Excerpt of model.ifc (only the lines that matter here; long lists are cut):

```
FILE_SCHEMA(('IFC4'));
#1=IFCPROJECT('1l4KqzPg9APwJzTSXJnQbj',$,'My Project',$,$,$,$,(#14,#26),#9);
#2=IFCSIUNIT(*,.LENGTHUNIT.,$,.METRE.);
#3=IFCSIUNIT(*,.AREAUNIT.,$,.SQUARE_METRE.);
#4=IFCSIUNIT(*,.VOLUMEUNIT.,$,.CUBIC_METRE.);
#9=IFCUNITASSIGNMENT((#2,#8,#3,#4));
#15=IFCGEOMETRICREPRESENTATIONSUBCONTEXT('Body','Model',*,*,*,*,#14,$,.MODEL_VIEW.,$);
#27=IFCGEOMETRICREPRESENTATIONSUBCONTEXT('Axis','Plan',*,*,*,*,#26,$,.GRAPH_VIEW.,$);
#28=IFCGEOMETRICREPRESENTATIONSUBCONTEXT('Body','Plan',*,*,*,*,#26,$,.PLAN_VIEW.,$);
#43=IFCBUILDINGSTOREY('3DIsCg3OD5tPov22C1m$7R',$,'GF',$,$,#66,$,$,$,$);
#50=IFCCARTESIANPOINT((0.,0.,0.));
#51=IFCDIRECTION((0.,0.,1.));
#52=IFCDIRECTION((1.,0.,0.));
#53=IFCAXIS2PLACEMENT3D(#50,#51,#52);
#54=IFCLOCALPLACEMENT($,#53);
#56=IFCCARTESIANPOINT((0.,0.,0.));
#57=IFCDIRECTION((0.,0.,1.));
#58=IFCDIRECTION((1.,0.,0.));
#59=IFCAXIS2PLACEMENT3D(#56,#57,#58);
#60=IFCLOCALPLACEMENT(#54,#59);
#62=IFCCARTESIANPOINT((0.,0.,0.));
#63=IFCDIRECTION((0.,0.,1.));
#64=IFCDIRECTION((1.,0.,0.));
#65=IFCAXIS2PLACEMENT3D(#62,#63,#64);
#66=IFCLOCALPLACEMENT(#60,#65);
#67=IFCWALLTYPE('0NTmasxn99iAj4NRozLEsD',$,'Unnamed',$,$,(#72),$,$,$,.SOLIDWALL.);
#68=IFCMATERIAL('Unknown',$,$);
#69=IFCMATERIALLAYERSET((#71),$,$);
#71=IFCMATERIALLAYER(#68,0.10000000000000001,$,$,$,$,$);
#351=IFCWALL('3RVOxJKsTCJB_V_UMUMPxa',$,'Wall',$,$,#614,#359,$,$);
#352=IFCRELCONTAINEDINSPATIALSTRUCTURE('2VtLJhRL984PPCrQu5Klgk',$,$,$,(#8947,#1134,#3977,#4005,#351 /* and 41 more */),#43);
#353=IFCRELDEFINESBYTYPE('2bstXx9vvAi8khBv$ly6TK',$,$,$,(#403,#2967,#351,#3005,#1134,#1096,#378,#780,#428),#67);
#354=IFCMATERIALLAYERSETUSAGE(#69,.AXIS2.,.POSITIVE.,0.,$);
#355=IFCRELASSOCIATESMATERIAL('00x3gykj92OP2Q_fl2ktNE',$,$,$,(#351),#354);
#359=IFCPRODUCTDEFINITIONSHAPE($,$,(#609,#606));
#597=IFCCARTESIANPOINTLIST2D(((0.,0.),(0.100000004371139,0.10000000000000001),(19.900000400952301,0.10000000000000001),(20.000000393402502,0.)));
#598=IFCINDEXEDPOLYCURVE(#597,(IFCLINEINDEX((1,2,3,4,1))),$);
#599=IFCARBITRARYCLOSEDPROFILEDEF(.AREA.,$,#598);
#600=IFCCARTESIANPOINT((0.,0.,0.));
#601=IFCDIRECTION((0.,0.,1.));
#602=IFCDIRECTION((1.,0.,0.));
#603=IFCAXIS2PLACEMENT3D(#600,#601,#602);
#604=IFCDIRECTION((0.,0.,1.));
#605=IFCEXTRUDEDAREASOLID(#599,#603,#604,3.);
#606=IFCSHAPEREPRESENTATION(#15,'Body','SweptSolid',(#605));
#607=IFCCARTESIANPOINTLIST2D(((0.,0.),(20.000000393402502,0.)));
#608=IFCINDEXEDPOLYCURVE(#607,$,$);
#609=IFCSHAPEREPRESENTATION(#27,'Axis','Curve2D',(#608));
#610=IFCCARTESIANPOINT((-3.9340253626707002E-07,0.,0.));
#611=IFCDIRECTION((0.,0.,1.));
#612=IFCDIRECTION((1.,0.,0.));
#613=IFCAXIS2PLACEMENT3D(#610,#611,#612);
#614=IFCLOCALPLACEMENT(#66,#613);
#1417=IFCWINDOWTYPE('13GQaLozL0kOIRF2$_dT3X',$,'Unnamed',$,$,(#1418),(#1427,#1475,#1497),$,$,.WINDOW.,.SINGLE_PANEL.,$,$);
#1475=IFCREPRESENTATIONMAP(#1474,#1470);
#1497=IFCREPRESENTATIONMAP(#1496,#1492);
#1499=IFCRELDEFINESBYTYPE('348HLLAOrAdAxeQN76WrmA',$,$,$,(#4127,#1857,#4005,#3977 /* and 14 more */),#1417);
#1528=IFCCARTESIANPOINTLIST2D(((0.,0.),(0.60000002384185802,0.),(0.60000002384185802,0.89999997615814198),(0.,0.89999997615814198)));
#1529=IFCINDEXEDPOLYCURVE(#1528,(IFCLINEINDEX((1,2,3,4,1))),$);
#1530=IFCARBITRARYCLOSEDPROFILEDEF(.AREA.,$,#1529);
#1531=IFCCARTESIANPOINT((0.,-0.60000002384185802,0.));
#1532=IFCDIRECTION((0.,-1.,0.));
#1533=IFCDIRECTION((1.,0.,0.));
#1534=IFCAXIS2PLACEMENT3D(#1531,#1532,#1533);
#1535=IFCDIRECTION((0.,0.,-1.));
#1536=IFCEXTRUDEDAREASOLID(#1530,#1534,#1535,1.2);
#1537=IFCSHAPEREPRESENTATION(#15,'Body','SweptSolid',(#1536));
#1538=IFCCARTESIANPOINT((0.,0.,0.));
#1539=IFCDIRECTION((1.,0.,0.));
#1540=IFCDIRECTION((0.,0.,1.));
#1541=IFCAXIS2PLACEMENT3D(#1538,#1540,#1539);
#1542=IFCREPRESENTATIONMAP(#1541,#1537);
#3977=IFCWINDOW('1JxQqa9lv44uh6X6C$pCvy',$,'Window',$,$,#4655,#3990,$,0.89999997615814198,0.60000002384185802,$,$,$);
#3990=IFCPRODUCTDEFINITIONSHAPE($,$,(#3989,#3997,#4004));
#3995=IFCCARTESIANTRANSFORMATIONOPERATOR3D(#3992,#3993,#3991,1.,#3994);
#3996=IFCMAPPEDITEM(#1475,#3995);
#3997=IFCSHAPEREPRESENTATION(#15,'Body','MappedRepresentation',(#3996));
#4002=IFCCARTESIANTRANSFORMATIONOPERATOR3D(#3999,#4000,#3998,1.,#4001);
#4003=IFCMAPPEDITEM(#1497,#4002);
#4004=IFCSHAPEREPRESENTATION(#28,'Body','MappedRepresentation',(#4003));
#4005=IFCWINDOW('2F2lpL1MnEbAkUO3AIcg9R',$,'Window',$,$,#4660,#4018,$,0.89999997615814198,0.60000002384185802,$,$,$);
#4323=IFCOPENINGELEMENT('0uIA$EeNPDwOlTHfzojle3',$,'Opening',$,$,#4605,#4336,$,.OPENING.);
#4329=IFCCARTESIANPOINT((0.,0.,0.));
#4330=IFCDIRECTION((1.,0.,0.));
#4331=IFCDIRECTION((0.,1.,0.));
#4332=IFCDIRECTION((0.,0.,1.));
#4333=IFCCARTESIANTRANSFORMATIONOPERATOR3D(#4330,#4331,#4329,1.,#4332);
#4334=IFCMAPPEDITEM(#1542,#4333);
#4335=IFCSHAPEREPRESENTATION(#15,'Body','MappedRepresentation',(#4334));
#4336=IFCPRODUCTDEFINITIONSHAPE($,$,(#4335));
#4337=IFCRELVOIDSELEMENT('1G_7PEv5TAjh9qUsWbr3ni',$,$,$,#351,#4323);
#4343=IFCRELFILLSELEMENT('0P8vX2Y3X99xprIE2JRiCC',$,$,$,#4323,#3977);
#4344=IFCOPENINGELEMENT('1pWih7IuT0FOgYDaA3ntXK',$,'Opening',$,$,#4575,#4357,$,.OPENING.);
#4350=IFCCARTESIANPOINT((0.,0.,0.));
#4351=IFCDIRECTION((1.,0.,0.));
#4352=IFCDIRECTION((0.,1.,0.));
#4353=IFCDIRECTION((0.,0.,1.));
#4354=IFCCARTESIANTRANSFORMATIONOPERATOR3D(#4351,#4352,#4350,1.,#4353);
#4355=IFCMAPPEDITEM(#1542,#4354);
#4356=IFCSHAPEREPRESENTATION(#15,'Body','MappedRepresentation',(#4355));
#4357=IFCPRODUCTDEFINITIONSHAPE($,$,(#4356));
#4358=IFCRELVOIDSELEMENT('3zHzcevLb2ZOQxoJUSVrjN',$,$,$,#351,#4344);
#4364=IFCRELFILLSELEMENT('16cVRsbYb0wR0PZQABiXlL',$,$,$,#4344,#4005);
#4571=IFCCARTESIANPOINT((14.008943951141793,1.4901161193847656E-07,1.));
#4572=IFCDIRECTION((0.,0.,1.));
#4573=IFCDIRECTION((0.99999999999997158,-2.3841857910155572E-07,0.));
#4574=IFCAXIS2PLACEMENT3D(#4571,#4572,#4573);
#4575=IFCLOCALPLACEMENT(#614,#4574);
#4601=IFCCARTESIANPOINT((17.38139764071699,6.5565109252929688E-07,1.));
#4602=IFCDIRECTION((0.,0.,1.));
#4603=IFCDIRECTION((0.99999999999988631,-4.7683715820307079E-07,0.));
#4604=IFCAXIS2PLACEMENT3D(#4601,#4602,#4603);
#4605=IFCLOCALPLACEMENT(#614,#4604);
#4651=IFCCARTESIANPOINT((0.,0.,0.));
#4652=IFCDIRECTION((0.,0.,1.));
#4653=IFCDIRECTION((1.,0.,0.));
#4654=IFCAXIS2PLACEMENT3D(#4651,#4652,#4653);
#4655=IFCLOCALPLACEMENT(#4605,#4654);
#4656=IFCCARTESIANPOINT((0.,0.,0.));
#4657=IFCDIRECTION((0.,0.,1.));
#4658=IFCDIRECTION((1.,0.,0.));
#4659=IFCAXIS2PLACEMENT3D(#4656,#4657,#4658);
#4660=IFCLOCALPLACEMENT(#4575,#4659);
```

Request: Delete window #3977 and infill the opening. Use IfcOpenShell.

```python
import ifcopenshell
import ifcopenshell.api.feature
import ifcopenshell.api.root
import ifcopenshell.geom
import ifcopenshell.util.shape

model = ifcopenshell.open("model.ifc")
settings = ifcopenshell.geom.settings()


def volume(element):
    """Net volume in cubic metres, openings subtracted."""
    shape = ifcopenshell.geom.create_shape(settings, element)
    return ifcopenshell.util.shape.get_volume(shape.geometry)


window = model.by_guid("1JxQqa9lv44uh6X6C$pCvy")
opening = window.FillsVoids[0].RelatingOpeningElement
wall = opening.VoidsElements[0].RelatingBuildingElement
before = volume(wall)

ifcopenshell.api.root.remove_product(model, product=window)
ifcopenshell.api.feature.remove_feature(model, feature=opening)

after = volume(wall)

print(f"wall volume {before:.3f} -> {after:.3f} m3")

model.write("model_v2.ifc")
```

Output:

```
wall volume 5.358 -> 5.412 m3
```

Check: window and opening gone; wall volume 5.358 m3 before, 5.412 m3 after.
